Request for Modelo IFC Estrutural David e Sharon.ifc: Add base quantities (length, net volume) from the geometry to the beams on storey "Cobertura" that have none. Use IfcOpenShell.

First a look at what the model holds.

```python
import ifcopenshell
import ifcopenshell.util.element
import ifcopenshell.util.unit

model = ifcopenshell.open("Modelo IFC Estrutural David e Sharon.ifc")
print(model.schema)
for unit_type in ("LENGTHUNIT", "AREAUNIT", "VOLUMEUNIT"):
    print(unit_type, ifcopenshell.util.unit.calculate_unit_scale(model, unit_type))
storey = next(s for s in model.by_type("IfcBuildingStorey") if s.Name == "Cobertura")
beams = [e for e in ifcopenshell.util.element.get_decomposition(storey) if e.is_a("IfcBeam")]
for e in sorted(beams, key=lambda e: e.id()):
    print(e.id(), e.is_a(), e.Name, list(ifcopenshell.util.element.get_psets(e, qtos_only=True)), sep=" | ")
```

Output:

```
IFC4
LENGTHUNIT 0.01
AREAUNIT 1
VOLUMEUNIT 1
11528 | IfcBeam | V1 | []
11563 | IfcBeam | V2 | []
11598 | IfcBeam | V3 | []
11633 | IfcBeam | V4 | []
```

```python
import ifcopenshell
import ifcopenshell.api.pset
import ifcopenshell.geom
import ifcopenshell.util.element
import ifcopenshell.util.shape
import ifcopenshell.util.unit

model = ifcopenshell.open("Modelo IFC Estrutural David e Sharon.ifc")
unit_scale = ifcopenshell.util.unit.calculate_unit_scale(model)
volume_scale = ifcopenshell.util.unit.calculate_unit_scale(model, "VOLUMEUNIT")
settings = ifcopenshell.geom.settings()

storey = next(s for s in model.by_type("IfcBuildingStorey") if s.Name == "Cobertura")
beams = [e for e in ifcopenshell.util.element.get_decomposition(storey) if e.is_a("IfcBeam")]

for e in sorted(beams, key=lambda e: e.id()):
    if ifcopenshell.util.element.get_psets(e, qtos_only=True, should_inherit=False):
        continue
    # Geometry comes back in metres, in the element's own axes.
    shape = ifcopenshell.geom.create_shape(settings, e)
    values = {
        "Length": ifcopenshell.util.shape.get_max_xyz(shape.geometry) / unit_scale,
        "NetVolume": ifcopenshell.util.shape.get_volume(shape.geometry) / volume_scale,
    }
    qto = ifcopenshell.api.pset.add_qto(model, product=e, name="Qto_BeamBaseQuantities")
    ifcopenshell.api.pset.edit_qto(model, qto=qto, properties=values)
    print(e.id(), {k: round(v, 3) for k, v in values.items()})

model.write("Modelo IFC Estrutural David e Sharon_updated.ifc")
```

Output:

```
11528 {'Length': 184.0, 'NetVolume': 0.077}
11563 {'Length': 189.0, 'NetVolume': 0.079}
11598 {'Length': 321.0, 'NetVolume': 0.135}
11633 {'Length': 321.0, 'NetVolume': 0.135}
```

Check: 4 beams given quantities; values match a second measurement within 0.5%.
